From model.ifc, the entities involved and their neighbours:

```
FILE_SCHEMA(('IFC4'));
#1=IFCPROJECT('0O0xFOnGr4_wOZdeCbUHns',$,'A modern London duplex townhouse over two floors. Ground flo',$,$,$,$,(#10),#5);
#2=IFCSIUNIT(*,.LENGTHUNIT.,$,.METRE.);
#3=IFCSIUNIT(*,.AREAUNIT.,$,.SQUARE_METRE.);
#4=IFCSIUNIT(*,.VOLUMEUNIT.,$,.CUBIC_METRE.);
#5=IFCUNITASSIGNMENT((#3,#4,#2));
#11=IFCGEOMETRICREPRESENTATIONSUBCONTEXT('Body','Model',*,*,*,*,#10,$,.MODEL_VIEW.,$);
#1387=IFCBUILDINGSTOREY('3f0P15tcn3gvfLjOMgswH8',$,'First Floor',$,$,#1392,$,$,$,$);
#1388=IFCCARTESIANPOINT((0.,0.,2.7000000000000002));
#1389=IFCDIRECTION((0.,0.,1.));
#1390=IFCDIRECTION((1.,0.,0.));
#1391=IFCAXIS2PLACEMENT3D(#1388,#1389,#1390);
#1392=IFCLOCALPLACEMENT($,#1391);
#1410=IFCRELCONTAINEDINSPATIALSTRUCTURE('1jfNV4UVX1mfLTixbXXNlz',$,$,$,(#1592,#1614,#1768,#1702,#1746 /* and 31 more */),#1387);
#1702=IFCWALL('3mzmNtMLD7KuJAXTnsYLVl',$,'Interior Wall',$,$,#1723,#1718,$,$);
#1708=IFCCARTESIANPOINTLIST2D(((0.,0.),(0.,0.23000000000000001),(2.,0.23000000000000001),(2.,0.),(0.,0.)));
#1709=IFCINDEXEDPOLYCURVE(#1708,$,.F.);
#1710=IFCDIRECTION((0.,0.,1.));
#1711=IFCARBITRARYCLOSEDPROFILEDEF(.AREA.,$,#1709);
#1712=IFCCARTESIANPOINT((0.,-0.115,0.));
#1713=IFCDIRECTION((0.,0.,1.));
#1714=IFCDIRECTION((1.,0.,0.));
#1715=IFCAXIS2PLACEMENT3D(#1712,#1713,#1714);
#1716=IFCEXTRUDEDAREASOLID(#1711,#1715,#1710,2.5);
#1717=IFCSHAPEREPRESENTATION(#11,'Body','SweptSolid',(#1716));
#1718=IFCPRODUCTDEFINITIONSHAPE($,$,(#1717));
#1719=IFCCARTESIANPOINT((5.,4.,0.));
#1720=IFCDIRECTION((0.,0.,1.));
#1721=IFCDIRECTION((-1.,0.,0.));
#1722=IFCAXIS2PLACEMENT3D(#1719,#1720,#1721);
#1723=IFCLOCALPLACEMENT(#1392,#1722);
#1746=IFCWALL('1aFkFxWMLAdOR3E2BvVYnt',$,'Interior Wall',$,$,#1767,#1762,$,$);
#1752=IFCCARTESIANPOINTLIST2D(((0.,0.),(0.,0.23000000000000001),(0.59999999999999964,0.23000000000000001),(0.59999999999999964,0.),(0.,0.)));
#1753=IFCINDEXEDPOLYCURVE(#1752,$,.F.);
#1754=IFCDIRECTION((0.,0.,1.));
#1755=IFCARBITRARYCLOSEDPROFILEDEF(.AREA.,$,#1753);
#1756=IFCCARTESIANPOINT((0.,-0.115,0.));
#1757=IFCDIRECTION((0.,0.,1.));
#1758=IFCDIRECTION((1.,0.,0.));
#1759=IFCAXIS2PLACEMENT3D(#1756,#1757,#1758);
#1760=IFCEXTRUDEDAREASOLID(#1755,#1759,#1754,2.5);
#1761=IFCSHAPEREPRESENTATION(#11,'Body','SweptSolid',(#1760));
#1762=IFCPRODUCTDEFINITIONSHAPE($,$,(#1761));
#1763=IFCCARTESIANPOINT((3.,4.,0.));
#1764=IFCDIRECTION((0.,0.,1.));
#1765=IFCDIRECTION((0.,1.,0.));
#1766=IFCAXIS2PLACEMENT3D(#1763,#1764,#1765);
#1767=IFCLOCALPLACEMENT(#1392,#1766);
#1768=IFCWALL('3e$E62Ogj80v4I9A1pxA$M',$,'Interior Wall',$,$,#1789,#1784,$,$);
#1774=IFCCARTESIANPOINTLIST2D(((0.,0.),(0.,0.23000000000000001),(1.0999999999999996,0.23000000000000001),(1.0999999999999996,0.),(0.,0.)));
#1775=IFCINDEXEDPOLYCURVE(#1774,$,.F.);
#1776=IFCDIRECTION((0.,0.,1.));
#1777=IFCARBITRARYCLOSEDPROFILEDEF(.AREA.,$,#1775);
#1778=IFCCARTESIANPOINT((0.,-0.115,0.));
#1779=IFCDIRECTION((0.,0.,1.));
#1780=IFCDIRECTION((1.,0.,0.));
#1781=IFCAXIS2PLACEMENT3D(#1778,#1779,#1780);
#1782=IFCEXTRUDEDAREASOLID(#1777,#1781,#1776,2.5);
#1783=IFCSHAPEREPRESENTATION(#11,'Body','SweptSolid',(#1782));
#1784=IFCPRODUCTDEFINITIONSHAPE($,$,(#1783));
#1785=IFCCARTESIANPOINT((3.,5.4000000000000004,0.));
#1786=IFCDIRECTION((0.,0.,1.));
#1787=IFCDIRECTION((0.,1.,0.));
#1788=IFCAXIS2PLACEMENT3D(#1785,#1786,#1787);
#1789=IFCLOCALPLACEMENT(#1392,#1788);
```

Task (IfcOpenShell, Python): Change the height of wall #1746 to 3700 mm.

```python
import ifcopenshell
import ifcopenshell.geom
import ifcopenshell.util.representation
import ifcopenshell.util.shape
import ifcopenshell.util.unit

model = ifcopenshell.open("model.ifc")
unit_scale = ifcopenshell.util.unit.calculate_unit_scale(model)
settings = ifcopenshell.geom.settings()


def volume(element):
    """Net volume in cubic metres, openings subtracted."""
    shape = ifcopenshell.geom.create_shape(settings, element)
    return ifcopenshell.util.shape.get_volume(shape.geometry)


wall = model.by_guid("1aFkFxWMLAdOR3E2BvVYnt")
before = volume(wall)

body = ifcopenshell.util.representation.get_representation(wall, "Model", "Body")
solid = body.Items[0]
old_height = solid.Depth
solid.Depth = 3.7 / unit_scale
after = volume(wall)

print(f"height {old_height:g} -> {solid.Depth:g}, volume {before:.3f} -> {after:.3f} m3")

model.write("model_edited.ifc")
```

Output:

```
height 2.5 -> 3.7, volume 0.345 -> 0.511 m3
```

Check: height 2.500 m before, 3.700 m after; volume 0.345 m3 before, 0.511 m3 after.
